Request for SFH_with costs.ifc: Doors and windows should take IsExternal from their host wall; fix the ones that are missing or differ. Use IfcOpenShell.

First a look at what the model holds.

```python
import ifcopenshell
import ifcopenshell.util.element

model = ifcopenshell.open("SFH_with costs.ifc")
print(model.schema)
seen = {}
for e in model.by_type("IfcDoor") + model.by_type("IfcWindow"):
    if not e.FillsVoids:
        continue
    host = e.FillsVoids[0].RelatingOpeningElement.VoidsElements[0].RelatingBuildingElement
    own = ifcopenshell.util.element.get_pset(e, f"Pset_{e.is_a()[3:].removesuffix('StandardCase')}Common", "IsExternal")
    wall = ifcopenshell.util.element.get_pset(host, "Pset_WallCommon", "IsExternal")
    seen[e.is_a(), own, wall] = seen.get((e.is_a(), own, wall), 0) + 1
for (cls, own, wall), count in sorted(seen.items(), key=str):
    print(count, cls, "IsExternal:", own, "| host wall:", wall)
```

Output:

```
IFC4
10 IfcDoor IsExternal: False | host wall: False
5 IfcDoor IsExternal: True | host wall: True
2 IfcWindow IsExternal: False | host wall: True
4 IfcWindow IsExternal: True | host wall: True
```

```python
import ifcopenshell
import ifcopenshell.api.pset
import ifcopenshell.util.element

model = ifcopenshell.open("SFH_with costs.ifc")

count = 0
for ifc_class, pset_name in (("IfcDoor", "Pset_DoorCommon"), ("IfcWindow", "Pset_WindowCommon")):
    for e in model.by_type(ifc_class):
        if not e.FillsVoids:
            continue
        host = e.FillsVoids[0].RelatingOpeningElement.VoidsElements[0].RelatingBuildingElement
        external = ifcopenshell.util.element.get_pset(host, "Pset_WallCommon", "IsExternal")
        if external is None or ifcopenshell.util.element.get_pset(e, pset_name, "IsExternal") == external:
            continue
        pset = ifcopenshell.api.pset.add_pset(model, product=e, name=pset_name)
        ifcopenshell.api.pset.edit_pset(model, pset=pset, properties={"IsExternal": external})
        count += 1

print(count, "updated")

model.write("SFH_with costs-out.ifc")
```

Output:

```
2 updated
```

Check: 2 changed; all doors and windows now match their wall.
